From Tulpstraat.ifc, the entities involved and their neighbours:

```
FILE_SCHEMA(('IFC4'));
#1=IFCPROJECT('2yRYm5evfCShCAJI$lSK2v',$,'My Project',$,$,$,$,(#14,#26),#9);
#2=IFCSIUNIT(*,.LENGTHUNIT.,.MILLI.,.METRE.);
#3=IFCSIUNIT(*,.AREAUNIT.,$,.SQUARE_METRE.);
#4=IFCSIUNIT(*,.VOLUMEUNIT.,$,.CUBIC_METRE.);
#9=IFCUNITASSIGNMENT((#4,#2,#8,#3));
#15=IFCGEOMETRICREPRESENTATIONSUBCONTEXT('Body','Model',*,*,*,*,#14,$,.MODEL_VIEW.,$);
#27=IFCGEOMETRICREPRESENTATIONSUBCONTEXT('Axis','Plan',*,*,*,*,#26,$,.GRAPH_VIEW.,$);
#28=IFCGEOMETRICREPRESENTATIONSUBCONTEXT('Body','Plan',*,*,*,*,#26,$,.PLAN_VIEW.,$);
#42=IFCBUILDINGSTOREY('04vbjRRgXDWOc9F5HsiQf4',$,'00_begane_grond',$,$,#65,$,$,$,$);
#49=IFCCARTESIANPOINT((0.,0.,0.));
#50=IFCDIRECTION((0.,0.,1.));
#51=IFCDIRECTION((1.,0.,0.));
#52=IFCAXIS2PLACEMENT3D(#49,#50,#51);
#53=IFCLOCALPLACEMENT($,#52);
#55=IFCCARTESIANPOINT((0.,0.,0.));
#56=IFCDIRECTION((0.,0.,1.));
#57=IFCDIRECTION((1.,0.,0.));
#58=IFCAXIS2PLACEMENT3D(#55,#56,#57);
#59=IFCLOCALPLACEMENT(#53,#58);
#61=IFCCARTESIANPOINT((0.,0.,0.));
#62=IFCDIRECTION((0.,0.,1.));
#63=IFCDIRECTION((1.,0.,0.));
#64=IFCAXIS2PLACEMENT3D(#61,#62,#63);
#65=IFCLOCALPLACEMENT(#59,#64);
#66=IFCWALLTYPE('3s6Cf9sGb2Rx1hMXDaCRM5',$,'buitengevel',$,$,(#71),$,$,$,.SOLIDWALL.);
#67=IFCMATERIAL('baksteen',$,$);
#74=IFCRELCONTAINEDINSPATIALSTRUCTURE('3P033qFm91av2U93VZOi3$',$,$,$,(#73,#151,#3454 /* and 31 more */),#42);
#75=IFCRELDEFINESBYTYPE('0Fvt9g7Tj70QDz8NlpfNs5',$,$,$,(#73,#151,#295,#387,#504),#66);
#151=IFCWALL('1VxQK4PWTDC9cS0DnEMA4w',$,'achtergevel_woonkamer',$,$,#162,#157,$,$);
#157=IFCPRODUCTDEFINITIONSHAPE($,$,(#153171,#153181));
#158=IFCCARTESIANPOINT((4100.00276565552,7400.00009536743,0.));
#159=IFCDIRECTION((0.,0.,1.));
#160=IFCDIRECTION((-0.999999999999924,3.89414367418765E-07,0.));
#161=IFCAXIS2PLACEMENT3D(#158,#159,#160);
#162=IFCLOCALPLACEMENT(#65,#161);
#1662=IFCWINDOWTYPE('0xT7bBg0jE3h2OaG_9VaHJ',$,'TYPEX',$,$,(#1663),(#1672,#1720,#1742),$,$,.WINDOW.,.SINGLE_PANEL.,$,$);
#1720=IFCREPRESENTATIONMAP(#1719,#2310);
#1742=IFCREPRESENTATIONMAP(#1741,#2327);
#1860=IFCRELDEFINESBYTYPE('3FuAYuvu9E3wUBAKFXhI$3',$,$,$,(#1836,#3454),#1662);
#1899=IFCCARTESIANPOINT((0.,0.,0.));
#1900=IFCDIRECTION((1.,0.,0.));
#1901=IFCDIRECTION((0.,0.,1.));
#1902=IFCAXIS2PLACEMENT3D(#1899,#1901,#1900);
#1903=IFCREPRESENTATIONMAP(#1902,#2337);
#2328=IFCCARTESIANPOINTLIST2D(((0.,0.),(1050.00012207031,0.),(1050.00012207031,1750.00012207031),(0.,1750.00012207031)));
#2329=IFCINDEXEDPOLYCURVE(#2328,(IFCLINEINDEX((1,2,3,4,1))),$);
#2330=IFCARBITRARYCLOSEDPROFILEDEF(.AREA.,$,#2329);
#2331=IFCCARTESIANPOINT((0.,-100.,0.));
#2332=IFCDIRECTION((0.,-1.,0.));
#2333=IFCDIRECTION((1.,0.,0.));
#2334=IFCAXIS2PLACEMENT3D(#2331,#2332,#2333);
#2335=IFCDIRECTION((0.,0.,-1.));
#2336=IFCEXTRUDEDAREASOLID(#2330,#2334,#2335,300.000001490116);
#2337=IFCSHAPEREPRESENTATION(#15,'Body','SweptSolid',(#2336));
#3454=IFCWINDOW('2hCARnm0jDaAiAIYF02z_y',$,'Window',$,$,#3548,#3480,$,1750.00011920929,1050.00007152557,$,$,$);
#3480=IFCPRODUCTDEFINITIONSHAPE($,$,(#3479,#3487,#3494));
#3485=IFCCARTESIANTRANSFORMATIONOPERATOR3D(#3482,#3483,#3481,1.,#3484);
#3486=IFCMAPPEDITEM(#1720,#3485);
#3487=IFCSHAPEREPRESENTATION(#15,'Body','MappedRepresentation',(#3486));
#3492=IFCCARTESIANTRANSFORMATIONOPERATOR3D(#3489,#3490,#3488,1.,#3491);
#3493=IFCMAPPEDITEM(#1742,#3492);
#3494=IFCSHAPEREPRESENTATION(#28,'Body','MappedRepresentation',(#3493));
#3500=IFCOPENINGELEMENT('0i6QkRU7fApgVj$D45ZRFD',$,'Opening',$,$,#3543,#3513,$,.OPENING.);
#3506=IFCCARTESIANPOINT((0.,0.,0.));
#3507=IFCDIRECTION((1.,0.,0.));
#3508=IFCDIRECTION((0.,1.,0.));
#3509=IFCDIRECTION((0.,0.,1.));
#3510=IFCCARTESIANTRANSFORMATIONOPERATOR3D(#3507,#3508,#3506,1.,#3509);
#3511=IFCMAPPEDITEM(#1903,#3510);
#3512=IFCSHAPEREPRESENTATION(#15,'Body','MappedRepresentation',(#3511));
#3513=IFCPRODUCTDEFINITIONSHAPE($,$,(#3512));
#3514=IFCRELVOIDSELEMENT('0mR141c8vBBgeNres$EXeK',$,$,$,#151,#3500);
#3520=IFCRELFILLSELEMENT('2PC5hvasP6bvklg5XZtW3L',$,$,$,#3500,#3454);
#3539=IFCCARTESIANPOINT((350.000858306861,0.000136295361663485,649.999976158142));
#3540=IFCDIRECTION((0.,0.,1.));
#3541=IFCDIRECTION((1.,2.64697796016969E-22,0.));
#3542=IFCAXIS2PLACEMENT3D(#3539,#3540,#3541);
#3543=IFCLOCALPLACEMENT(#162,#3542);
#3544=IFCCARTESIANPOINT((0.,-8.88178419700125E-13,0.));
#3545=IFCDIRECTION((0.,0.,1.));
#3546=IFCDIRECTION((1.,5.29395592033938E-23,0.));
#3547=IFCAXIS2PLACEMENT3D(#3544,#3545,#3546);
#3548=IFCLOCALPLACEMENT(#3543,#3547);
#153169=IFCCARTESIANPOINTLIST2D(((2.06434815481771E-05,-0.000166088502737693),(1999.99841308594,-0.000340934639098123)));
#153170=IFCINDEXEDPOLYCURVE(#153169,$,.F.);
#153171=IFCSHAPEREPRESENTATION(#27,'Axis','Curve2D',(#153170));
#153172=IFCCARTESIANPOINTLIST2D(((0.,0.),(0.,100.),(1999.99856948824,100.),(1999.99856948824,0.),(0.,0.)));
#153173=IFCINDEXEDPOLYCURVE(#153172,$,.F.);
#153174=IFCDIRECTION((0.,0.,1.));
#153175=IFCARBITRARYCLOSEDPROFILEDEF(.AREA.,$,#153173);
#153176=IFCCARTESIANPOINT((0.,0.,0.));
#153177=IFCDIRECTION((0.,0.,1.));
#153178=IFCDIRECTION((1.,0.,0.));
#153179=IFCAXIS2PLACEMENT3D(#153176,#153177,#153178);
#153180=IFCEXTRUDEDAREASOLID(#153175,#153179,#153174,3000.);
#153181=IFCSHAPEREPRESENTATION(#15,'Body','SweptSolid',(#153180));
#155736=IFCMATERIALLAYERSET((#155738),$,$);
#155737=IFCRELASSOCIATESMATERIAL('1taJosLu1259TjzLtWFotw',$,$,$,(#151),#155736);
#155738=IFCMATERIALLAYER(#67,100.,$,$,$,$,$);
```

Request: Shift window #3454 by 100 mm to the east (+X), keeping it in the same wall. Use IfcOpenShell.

```python
import ifcopenshell
import ifcopenshell.api.geometry
import ifcopenshell.util.placement
import ifcopenshell.util.unit

model = ifcopenshell.open("Tulpstraat.ifc")
unit_scale = ifcopenshell.util.unit.calculate_unit_scale(model)

window = model.by_guid("2hCARnm0jDaAiAIYF02z_y")
opening = window.FillsVoids[0].RelatingOpeningElement
wall = opening.VoidsElements[0].RelatingBuildingElement

wall_matrix = ifcopenshell.util.placement.get_local_placement(wall.ObjectPlacement)
shift = wall_matrix[:3, 0] * -0.1 / unit_scale
before = ifcopenshell.util.placement.get_local_placement(window.ObjectPlacement)[:3, 3].copy()

# The window is placed relative to its opening, so it follows when the opening moves.
matrix = ifcopenshell.util.placement.get_local_placement(opening.ObjectPlacement)
matrix[:3, 3] += shift
ifcopenshell.api.geometry.edit_object_placement(
    model, product=opening, matrix=matrix, is_si=False, should_transform_children=True
)

after = ifcopenshell.util.placement.get_local_placement(window.ObjectPlacement)[:3, 3]
print("window moved by", (after - before).round(3) + 0.0)

model.write("Tulpstraat_rev.ifc")
```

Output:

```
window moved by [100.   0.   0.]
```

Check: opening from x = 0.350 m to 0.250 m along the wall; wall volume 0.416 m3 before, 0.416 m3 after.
